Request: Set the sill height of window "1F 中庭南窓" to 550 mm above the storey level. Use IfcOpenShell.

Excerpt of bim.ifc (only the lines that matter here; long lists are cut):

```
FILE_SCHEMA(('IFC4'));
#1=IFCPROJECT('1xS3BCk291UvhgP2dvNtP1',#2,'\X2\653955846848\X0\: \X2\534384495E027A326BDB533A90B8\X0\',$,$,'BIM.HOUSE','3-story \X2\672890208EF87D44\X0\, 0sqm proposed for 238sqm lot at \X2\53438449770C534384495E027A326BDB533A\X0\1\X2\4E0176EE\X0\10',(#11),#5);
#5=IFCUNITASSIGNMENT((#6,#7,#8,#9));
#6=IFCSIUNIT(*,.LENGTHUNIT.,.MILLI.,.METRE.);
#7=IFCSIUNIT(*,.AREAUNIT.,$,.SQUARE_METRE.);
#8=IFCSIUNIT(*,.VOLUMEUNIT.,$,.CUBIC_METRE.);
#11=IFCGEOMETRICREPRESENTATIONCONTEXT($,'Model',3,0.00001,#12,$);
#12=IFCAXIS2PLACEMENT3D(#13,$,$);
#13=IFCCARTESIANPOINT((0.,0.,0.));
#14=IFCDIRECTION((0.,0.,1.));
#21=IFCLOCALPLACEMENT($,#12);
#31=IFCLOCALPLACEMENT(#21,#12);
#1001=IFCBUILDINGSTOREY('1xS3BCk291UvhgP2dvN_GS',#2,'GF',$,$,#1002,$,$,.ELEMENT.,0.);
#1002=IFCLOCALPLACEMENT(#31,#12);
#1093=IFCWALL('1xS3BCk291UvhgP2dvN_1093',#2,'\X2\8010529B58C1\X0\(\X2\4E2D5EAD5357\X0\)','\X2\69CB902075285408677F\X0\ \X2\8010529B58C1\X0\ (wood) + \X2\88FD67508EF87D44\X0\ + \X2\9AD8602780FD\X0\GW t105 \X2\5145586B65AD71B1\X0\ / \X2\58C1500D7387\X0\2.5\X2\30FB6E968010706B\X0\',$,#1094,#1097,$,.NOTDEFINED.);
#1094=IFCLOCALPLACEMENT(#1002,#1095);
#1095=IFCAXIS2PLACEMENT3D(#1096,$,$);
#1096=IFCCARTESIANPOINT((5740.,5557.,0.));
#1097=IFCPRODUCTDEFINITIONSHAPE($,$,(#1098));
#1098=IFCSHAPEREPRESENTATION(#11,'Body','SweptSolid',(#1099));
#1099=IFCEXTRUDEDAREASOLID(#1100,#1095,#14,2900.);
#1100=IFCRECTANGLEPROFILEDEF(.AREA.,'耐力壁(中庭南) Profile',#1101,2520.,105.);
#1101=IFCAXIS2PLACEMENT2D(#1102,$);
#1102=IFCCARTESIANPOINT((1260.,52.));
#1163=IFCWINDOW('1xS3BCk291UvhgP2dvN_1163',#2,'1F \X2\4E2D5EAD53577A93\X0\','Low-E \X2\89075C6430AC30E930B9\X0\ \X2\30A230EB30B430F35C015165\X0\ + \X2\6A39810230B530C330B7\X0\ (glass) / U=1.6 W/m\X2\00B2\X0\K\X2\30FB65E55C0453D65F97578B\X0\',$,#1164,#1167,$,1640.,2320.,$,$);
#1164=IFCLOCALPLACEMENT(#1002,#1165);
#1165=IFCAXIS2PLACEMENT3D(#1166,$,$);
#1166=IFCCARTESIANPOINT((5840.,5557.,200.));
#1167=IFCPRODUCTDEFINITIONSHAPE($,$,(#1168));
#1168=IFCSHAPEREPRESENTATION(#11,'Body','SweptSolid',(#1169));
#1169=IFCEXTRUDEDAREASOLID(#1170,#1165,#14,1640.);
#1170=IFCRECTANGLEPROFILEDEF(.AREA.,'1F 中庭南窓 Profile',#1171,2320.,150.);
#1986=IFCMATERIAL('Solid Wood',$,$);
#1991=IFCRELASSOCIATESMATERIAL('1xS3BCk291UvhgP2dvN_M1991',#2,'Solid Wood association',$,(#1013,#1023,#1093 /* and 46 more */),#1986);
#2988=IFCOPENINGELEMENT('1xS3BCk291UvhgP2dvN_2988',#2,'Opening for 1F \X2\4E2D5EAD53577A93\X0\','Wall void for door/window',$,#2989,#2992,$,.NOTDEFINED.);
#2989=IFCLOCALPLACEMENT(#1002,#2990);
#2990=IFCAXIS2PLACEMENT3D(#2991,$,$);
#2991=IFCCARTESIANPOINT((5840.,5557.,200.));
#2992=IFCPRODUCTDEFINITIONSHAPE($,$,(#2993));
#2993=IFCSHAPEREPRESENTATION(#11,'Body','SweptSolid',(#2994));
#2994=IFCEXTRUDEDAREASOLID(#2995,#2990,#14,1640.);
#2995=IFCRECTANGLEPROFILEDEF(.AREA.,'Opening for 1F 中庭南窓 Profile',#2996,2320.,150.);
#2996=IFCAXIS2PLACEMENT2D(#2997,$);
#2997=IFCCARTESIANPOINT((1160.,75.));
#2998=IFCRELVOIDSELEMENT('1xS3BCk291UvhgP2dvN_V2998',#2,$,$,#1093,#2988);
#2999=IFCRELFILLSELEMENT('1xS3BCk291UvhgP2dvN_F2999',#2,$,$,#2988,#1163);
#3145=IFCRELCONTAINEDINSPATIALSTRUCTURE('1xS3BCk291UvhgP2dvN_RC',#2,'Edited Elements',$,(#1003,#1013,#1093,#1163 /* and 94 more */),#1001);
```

```python
import numpy as np
import ifcopenshell
import ifcopenshell.api.geometry
import ifcopenshell.geom
import ifcopenshell.util.element
import ifcopenshell.util.placement
import ifcopenshell.util.shape
import ifcopenshell.util.unit

model = ifcopenshell.open("bim.ifc")
unit_scale = ifcopenshell.util.unit.calculate_unit_scale(model)

window = model.by_id(1163)
opening = window.FillsVoids[0].RelatingOpeningElement
storey = ifcopenshell.util.element.get_container(window, ifc_class="IfcBuildingStorey")
level = ifcopenshell.util.placement.get_local_placement(storey.ObjectPlacement)[2, 3]

# The opening's origin need not be at the sill, so measure its lowest point.
shape = ifcopenshell.geom.create_shape(ifcopenshell.geom.settings(), opening)
bottom = ifcopenshell.util.shape.get_shape_bottom_elevation(shape, shape.geometry) / unit_scale
dz = level + 550.0 - bottom

shift = np.array([0.0, 0.0, dz])
# The window is not placed relative to its opening, so move both.
for product in (opening, window):
    matrix = ifcopenshell.util.placement.get_local_placement(product.ObjectPlacement)
    matrix[:3, 3] += shift
    ifcopenshell.api.geometry.edit_object_placement(model, product=product, matrix=matrix, is_si=False)

print(f"moved by {dz * unit_scale:+.3f} m")

model.write("bim_rev.ifc")
```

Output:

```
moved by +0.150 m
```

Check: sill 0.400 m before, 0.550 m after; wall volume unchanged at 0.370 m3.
